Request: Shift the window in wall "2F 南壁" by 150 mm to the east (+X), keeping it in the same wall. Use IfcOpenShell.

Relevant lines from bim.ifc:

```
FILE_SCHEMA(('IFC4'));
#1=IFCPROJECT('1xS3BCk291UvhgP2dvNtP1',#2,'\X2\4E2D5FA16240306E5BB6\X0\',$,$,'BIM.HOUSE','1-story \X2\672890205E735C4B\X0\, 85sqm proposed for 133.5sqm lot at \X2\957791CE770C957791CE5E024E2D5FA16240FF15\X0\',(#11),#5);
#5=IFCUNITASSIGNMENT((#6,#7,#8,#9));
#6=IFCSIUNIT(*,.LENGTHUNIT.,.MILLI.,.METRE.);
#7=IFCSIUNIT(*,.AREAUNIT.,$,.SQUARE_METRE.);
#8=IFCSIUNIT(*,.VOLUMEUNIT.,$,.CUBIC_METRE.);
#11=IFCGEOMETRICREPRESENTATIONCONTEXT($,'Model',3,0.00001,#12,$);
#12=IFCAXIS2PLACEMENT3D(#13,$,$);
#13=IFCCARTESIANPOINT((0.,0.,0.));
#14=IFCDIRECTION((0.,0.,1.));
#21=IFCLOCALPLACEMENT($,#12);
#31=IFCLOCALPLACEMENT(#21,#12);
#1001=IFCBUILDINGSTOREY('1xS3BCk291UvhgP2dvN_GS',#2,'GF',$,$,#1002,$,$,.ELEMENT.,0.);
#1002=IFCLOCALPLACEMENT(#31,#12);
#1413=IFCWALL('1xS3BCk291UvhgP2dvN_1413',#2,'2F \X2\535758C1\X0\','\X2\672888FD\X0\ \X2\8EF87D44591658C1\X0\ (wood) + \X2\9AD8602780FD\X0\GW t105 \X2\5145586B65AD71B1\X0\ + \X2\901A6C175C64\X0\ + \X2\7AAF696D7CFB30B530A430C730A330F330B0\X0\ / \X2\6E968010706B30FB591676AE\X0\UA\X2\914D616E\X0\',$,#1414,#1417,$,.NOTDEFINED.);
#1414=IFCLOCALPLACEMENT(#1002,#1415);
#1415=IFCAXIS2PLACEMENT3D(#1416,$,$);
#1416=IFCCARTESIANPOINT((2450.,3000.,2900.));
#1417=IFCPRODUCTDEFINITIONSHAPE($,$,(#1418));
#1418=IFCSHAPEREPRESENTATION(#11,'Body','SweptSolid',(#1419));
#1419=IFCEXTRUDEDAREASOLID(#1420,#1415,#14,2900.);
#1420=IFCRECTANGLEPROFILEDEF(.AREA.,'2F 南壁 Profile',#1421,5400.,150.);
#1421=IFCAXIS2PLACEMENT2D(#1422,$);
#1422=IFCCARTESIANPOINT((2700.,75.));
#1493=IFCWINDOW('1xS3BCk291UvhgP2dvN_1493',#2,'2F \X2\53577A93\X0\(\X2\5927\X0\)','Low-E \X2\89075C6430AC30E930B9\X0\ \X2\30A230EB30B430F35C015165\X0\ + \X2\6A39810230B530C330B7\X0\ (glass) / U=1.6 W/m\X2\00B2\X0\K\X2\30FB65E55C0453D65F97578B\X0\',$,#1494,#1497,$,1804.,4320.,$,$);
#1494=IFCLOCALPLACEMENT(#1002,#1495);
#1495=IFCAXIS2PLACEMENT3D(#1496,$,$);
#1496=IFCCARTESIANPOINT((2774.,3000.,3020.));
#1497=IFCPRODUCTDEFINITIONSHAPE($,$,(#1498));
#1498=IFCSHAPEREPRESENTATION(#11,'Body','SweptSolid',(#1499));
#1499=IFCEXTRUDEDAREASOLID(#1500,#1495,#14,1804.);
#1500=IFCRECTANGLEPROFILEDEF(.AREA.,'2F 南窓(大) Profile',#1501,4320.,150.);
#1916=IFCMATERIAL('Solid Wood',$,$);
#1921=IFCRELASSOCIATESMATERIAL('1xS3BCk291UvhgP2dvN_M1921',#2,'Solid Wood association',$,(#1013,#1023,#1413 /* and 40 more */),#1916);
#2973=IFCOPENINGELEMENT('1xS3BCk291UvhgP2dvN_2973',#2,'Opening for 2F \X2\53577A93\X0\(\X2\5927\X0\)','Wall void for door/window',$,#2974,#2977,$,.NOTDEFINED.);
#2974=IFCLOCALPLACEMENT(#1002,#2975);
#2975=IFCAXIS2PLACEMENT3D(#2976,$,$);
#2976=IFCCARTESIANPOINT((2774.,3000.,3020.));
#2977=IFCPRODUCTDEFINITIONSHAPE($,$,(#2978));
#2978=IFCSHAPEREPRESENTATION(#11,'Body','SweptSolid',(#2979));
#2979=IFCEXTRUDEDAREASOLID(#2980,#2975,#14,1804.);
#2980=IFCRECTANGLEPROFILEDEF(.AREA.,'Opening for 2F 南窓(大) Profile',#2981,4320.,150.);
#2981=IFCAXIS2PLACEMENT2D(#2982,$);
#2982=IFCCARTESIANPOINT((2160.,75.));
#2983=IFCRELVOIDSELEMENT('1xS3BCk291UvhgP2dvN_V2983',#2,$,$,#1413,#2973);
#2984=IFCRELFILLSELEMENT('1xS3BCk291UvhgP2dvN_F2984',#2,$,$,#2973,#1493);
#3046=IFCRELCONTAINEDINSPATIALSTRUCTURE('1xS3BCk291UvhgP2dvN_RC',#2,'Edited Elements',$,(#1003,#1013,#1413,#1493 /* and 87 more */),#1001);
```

```python
import ifcopenshell
import ifcopenshell.api.geometry
import ifcopenshell.util.placement

model = ifcopenshell.open("bim.ifc")

window = model.by_guid("1xS3BCk291UvhgP2dvN_1493")
opening = window.FillsVoids[0].RelatingOpeningElement
wall = opening.VoidsElements[0].RelatingBuildingElement

wall_matrix = ifcopenshell.util.placement.get_local_placement(wall.ObjectPlacement)
shift = wall_matrix[:3, 0] * 150.0
before = ifcopenshell.util.placement.get_local_placement(window.ObjectPlacement)[:3, 3].copy()

# The window is not placed relative to its opening, so move both.
for product in (opening, window):
    matrix = ifcopenshell.util.placement.get_local_placement(product.ObjectPlacement)
    matrix[:3, 3] += shift
    ifcopenshell.api.geometry.edit_object_placement(model, product=product, matrix=matrix, is_si=False)

after = ifcopenshell.util.placement.get_local_placement(window.ObjectPlacement)[:3, 3]
print("window moved by", (after - before).round(3) + 0.0)

model.write("bim_updated.ifc")
```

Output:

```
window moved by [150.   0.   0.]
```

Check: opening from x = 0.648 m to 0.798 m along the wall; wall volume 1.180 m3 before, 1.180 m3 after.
